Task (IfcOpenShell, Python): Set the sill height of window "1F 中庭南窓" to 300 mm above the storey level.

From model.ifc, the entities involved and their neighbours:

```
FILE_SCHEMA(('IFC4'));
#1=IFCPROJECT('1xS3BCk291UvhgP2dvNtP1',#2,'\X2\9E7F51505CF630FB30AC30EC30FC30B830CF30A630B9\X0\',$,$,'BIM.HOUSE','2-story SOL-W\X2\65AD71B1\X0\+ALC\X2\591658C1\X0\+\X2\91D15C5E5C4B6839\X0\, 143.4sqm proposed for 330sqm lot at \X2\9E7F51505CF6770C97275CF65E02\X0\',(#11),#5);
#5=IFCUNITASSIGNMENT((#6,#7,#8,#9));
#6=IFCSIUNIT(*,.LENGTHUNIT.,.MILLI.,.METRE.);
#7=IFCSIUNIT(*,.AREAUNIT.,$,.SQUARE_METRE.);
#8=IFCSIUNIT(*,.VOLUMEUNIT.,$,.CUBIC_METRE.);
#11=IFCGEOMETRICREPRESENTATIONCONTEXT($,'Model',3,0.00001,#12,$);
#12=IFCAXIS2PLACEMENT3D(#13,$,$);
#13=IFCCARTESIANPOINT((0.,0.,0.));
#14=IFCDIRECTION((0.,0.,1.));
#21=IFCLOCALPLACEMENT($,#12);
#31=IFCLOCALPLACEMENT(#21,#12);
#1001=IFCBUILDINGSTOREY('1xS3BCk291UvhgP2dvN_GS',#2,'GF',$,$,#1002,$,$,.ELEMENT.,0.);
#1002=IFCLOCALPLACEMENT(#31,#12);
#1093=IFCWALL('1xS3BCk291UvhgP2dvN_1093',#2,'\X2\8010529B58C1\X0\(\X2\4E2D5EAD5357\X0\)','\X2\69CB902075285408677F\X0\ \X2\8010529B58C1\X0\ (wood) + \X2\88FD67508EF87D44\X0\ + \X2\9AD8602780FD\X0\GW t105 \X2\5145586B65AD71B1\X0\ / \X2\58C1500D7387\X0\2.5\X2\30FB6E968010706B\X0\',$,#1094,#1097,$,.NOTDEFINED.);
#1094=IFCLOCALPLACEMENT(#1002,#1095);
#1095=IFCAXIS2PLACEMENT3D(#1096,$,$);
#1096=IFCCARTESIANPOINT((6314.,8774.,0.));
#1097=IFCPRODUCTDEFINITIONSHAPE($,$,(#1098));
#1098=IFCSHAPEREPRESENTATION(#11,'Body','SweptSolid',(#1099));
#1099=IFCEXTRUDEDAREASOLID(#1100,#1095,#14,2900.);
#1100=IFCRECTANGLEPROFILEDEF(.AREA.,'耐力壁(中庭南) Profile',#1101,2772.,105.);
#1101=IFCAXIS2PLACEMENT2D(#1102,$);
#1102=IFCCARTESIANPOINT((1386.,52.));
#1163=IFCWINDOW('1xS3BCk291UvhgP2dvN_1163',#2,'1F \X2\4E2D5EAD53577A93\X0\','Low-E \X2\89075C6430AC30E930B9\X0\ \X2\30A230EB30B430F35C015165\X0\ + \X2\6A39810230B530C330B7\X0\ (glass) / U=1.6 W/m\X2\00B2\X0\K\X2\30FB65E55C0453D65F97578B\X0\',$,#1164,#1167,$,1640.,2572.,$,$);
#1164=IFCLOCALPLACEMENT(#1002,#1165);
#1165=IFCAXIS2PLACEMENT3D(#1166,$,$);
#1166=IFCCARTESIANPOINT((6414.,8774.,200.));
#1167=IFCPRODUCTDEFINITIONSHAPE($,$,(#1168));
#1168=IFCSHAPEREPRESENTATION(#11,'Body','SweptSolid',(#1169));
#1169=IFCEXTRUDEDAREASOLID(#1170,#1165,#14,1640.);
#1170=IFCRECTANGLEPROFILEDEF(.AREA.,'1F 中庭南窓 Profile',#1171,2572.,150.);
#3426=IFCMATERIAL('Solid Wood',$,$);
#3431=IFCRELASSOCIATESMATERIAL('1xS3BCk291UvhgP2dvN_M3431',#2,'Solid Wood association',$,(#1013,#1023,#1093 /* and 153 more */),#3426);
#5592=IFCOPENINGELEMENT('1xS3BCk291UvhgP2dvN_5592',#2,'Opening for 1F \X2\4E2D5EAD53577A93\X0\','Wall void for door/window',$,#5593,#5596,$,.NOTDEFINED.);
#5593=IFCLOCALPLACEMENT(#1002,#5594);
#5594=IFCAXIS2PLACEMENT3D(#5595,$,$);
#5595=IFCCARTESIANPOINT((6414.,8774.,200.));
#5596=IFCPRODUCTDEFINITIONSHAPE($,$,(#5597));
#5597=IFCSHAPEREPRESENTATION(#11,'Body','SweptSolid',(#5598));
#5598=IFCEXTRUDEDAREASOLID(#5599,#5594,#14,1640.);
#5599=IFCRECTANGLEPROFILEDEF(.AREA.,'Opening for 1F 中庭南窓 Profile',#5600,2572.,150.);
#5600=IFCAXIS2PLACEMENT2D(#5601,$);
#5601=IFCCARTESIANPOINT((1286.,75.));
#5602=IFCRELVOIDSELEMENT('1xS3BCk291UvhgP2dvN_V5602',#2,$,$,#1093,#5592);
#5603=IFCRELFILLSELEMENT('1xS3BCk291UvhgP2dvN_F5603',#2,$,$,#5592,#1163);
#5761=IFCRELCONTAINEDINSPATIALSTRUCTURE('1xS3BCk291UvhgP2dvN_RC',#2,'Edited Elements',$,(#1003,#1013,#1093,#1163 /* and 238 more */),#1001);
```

```python
import numpy as np
import ifcopenshell
import ifcopenshell.api.geometry
import ifcopenshell.geom
import ifcopenshell.util.element
import ifcopenshell.util.placement
import ifcopenshell.util.shape
import ifcopenshell.util.unit

model = ifcopenshell.open("model.ifc")
unit_scale = ifcopenshell.util.unit.calculate_unit_scale(model)

window = model.by_guid("1xS3BCk291UvhgP2dvN_1163")
opening = window.FillsVoids[0].RelatingOpeningElement
storey = ifcopenshell.util.element.get_container(window, ifc_class="IfcBuildingStorey")
level = ifcopenshell.util.placement.get_local_placement(storey.ObjectPlacement)[2, 3]

# The opening's origin need not be at the sill, so measure its lowest point.
shape = ifcopenshell.geom.create_shape(ifcopenshell.geom.settings(), opening)
bottom = ifcopenshell.util.shape.get_shape_bottom_elevation(shape, shape.geometry) / unit_scale
dz = level + 0.3 / unit_scale - bottom

shift = np.array([0.0, 0.0, dz])
# The window is not placed relative to its opening, so move both.
for product in (opening, window):
    matrix = ifcopenshell.util.placement.get_local_placement(product.ObjectPlacement)
    matrix[:3, 3] += shift
    ifcopenshell.api.geometry.edit_object_placement(model, product=product, matrix=matrix, is_si=False)

print(f"moved by {dz * unit_scale:+.3f} m")

model.write("model_updated.ifc")
```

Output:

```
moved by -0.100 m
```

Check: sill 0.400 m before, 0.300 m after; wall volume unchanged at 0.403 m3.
